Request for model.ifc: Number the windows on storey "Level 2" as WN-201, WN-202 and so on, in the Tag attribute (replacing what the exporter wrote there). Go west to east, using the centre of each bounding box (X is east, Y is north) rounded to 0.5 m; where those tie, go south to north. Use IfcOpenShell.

First a look at what the model holds.

```python
import ifcopenshell
import ifcopenshell.util.element
import ifcopenshell.util.placement

model = ifcopenshell.open("model.ifc")
print(model.schema)
storey = next(s for s in model.by_type("IfcBuildingStorey") if s.Name == "Level 2")
windows = [e for e in ifcopenshell.util.element.get_decomposition(storey) if e.is_a("IfcWindow")]
for e in sorted(windows, key=lambda e: e.id()):
    origin = ifcopenshell.util.placement.get_local_placement(e.ObjectPlacement)[:3, 3]
    print(e.id(), e.Tag, e.Name, origin.round(2) + 0.0, sep=" | ")
```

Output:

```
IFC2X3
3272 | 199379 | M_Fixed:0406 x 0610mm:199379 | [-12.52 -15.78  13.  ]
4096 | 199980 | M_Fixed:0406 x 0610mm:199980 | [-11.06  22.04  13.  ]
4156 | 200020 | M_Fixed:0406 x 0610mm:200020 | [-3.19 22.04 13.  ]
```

```python
import ifcopenshell
import ifcopenshell.geom
import ifcopenshell.util.element
import ifcopenshell.util.shape

model = ifcopenshell.open("model.ifc")
settings = ifcopenshell.geom.settings()
settings.set("use-world-coords", True)


def centre(element):
    shape = ifcopenshell.geom.create_shape(settings, element)
    return ifcopenshell.util.shape.get_bbox_centroid(shape.geometry)


storey = next(s for s in model.by_type("IfcBuildingStorey") if s.Name == "Level 2")
windows = [e for e in ifcopenshell.util.element.get_decomposition(storey) if e.is_a("IfcWindow")]

# Insertion points can sit at a corner or the storey origin, so sort by the geometry (in metres).
centres = {e: centre(e) for e in windows}
windows.sort(key=lambda e: (round(centres[e][0] / 0.5), centres[e][1]))

for i, e in enumerate(windows, start=1):
    number = f"WN-2{i:02d}"
    e.Tag = number
    print(e.id(), number)

model.write("model_edited.ifc")
```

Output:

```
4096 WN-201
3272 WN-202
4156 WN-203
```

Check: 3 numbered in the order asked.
